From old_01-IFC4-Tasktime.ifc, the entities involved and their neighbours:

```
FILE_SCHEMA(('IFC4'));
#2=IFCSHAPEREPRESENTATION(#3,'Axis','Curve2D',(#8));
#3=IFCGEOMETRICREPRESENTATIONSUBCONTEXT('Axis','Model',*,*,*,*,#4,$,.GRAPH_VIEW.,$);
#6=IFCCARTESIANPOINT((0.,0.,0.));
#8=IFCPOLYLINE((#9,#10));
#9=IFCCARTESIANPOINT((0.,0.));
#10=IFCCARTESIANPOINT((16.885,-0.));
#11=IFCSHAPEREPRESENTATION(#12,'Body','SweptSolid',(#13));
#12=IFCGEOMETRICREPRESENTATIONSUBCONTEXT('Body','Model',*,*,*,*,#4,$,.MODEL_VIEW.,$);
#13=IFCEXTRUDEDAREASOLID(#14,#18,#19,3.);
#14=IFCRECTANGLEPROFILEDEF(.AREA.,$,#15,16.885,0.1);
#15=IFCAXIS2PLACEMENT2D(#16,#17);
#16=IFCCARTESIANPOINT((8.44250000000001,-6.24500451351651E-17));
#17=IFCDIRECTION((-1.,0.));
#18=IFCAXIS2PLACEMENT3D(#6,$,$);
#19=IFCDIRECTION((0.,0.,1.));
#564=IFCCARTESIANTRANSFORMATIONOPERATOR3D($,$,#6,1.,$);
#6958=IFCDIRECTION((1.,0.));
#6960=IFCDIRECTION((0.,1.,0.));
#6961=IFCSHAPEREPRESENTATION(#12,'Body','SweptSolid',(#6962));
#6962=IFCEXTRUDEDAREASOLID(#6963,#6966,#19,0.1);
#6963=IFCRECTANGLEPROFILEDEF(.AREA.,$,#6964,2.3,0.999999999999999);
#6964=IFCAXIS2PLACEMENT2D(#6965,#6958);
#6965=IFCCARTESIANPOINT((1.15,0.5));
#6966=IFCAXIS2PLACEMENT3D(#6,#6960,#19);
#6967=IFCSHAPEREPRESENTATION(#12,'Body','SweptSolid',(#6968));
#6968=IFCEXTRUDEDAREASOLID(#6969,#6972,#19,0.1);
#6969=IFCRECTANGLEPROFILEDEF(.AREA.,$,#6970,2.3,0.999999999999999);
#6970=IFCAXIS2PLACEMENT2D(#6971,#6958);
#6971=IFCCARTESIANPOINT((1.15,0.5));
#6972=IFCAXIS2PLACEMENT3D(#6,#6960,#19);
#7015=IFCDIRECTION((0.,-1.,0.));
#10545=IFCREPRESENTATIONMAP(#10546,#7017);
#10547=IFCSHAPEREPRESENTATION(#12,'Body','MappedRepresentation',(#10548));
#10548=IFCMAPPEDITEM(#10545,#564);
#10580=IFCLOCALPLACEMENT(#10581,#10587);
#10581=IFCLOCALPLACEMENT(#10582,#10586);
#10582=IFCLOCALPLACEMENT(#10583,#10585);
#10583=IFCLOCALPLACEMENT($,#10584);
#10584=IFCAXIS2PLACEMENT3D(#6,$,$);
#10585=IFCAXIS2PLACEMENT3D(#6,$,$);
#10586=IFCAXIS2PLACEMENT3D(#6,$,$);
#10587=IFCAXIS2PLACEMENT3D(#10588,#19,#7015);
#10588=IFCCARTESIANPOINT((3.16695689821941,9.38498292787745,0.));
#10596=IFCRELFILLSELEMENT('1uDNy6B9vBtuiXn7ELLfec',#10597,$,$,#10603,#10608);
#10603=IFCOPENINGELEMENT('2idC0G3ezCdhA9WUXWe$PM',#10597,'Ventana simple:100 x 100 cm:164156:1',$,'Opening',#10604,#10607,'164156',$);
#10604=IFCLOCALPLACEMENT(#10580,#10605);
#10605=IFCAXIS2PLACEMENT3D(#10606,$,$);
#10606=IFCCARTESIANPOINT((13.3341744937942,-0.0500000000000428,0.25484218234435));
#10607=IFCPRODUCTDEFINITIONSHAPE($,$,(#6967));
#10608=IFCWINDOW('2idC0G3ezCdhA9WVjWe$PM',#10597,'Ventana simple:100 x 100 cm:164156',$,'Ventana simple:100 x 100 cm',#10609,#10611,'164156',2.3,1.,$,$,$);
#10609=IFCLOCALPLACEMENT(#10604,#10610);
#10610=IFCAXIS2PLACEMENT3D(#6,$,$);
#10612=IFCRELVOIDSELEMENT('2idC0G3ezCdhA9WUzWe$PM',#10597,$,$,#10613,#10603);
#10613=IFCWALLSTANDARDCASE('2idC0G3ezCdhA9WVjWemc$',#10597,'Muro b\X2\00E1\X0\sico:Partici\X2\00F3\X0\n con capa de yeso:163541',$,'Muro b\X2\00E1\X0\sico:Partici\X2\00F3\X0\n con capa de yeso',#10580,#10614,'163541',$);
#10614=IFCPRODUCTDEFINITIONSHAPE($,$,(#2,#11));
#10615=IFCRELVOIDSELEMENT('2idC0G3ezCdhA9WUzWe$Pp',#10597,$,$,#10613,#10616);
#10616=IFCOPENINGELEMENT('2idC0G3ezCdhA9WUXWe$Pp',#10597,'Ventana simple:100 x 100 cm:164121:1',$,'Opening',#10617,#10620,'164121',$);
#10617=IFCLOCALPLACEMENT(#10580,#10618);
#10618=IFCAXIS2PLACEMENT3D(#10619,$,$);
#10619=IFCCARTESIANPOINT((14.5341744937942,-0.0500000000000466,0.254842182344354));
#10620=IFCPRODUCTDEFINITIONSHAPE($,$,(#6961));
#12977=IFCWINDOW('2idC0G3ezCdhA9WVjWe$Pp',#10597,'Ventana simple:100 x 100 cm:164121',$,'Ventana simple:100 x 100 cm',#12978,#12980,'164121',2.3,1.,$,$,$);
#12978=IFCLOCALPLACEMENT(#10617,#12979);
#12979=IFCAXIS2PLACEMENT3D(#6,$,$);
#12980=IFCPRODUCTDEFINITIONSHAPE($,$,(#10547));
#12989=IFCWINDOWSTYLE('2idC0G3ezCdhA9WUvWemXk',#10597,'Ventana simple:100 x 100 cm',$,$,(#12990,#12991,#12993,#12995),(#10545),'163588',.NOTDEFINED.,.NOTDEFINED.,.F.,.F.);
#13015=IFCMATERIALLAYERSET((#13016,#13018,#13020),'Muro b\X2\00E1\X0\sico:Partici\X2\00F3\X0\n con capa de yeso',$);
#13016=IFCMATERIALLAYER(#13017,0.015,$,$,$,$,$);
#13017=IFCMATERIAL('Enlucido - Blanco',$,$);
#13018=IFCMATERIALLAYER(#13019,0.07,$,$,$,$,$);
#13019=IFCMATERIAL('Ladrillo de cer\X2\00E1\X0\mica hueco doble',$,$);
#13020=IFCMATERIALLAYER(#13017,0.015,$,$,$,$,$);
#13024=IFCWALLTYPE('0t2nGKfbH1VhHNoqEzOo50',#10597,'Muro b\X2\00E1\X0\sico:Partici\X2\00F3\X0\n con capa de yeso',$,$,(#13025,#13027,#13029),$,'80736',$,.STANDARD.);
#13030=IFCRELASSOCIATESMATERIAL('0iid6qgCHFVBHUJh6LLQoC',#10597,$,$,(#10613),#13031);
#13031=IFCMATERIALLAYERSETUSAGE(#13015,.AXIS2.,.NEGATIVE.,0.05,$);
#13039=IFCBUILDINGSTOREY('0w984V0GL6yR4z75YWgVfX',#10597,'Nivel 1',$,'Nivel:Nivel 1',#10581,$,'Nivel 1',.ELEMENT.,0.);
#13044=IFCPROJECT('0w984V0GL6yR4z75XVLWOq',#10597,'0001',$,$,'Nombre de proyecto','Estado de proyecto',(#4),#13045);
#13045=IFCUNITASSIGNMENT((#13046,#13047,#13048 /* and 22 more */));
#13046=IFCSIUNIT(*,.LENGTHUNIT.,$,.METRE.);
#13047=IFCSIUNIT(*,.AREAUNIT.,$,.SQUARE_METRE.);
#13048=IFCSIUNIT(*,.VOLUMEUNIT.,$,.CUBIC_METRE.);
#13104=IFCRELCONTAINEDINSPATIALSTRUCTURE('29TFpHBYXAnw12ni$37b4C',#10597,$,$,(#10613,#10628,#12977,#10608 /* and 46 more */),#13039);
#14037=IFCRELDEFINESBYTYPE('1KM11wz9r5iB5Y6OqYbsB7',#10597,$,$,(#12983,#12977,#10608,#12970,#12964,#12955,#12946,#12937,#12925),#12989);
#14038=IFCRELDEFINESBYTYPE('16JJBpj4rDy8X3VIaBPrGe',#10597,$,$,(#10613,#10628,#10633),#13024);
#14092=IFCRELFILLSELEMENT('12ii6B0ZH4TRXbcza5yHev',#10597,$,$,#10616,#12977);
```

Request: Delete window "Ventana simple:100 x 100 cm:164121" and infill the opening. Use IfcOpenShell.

```python
import ifcopenshell
import ifcopenshell.api.feature
import ifcopenshell.api.root
import ifcopenshell.geom
import ifcopenshell.util.shape

model = ifcopenshell.open("old_01-IFC4-Tasktime.ifc")
settings = ifcopenshell.geom.settings()


def volume(element):
    """Net volume in cubic metres, openings subtracted."""
    shape = ifcopenshell.geom.create_shape(settings, element)
    return ifcopenshell.util.shape.get_volume(shape.geometry)


window = model.by_guid("2idC0G3ezCdhA9WVjWe$Pp")
opening = window.FillsVoids[0].RelatingOpeningElement
wall = opening.VoidsElements[0].RelatingBuildingElement
before = volume(wall)

ifcopenshell.api.root.remove_product(model, product=window)
ifcopenshell.api.feature.remove_feature(model, feature=opening)

after = volume(wall)

print(f"wall volume {before:.3f} -> {after:.3f} m3")

model.write("old_01-IFC4-Tasktime-out.ifc")
```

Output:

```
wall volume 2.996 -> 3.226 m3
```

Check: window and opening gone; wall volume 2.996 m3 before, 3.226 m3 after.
